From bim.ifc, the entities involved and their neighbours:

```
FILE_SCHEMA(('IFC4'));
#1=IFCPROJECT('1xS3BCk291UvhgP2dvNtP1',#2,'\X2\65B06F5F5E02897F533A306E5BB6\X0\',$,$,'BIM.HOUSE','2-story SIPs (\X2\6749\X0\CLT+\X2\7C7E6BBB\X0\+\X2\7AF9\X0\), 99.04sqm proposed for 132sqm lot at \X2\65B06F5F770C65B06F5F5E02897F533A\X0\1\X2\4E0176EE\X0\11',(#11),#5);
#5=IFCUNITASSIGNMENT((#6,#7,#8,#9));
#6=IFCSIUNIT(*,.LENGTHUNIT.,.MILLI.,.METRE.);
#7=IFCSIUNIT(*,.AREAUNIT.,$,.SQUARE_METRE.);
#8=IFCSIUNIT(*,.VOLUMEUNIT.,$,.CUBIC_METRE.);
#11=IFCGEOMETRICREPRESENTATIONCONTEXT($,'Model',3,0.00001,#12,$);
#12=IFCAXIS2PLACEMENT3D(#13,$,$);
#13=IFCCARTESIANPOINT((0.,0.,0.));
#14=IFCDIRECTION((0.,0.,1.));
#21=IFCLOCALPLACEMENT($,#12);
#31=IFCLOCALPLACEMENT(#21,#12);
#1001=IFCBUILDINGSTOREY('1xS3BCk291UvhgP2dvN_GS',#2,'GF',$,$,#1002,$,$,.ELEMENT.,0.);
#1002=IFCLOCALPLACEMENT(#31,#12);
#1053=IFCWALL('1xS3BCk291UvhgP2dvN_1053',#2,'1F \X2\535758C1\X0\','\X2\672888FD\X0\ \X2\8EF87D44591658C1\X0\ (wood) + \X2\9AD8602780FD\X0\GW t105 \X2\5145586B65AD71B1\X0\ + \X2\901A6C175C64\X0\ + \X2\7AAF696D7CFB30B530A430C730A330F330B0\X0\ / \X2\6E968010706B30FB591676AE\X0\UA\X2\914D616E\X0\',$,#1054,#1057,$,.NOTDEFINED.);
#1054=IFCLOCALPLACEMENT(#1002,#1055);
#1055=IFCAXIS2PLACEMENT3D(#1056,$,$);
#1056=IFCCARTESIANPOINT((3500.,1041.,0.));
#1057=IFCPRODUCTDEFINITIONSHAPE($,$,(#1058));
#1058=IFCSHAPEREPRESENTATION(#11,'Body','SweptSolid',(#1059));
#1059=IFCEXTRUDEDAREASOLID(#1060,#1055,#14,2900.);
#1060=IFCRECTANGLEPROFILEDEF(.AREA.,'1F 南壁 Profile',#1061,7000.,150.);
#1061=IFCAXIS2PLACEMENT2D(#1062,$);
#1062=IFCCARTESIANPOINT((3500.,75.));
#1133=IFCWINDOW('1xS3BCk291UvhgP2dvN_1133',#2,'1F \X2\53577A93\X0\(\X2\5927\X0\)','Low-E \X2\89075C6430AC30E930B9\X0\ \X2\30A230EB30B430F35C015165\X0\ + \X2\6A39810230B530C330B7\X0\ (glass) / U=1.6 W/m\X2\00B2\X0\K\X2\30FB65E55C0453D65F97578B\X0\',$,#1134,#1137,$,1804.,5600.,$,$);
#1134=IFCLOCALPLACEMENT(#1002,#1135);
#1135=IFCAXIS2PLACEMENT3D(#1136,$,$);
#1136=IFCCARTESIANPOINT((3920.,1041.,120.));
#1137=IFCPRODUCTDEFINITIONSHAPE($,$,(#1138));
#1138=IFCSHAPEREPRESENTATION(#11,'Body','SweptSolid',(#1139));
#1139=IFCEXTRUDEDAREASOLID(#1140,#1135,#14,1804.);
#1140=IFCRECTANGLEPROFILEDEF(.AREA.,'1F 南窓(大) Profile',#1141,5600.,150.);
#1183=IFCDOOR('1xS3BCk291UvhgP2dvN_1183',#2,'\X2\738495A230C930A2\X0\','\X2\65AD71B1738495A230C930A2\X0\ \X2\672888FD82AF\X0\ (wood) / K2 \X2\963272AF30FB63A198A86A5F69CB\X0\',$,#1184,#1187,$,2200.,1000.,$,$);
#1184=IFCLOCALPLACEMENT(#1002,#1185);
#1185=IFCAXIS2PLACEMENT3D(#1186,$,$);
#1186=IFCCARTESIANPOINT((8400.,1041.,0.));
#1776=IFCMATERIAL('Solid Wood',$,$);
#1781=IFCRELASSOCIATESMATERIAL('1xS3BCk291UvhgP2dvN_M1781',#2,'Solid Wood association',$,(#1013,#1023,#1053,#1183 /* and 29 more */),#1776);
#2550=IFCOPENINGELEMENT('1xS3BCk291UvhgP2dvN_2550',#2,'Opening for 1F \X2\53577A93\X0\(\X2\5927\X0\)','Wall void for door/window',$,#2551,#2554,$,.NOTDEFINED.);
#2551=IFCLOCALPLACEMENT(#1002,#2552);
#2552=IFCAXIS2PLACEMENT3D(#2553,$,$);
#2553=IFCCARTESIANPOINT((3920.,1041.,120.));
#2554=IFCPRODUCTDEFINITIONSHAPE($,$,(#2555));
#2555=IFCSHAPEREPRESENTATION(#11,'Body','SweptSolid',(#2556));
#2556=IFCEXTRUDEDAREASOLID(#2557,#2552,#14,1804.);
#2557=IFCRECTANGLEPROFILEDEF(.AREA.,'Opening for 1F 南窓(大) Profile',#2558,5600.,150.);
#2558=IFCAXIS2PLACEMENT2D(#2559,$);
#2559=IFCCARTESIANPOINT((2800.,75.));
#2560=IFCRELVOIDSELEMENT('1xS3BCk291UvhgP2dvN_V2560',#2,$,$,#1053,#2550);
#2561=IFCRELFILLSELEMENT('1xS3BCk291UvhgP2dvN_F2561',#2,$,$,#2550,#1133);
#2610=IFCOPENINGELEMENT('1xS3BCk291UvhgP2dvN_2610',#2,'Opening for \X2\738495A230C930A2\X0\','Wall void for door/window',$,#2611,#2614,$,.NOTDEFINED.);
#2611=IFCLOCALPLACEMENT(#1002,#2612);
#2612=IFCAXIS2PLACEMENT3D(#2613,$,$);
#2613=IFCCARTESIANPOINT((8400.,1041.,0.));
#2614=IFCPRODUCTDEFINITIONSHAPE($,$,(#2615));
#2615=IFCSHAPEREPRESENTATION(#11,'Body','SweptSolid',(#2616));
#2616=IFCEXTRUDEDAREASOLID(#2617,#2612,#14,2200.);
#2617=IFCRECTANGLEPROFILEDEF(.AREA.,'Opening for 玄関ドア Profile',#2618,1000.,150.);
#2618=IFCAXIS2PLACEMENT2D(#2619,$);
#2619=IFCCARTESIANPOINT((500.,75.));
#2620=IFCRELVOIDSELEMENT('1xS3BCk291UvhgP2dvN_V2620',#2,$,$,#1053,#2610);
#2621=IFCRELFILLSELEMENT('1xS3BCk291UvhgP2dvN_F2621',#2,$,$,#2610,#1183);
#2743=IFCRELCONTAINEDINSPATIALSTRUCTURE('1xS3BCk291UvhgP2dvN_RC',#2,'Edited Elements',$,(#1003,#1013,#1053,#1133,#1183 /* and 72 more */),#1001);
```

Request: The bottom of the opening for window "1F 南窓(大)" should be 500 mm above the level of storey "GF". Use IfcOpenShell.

```python
import numpy as np
import ifcopenshell
import ifcopenshell.api.geometry
import ifcopenshell.geom
import ifcopenshell.util.element
import ifcopenshell.util.placement
import ifcopenshell.util.shape
import ifcopenshell.util.unit

model = ifcopenshell.open("bim.ifc")
unit_scale = ifcopenshell.util.unit.calculate_unit_scale(model)

window = model.by_guid("1xS3BCk291UvhgP2dvN_1133")
opening = window.FillsVoids[0].RelatingOpeningElement
storey = ifcopenshell.util.element.get_container(window, ifc_class="IfcBuildingStorey")
level = ifcopenshell.util.placement.get_local_placement(storey.ObjectPlacement)[2, 3]

# The opening's origin need not be at the sill, so measure its lowest point.
shape = ifcopenshell.geom.create_shape(ifcopenshell.geom.settings(), opening)
bottom = ifcopenshell.util.shape.get_shape_bottom_elevation(shape, shape.geometry) / unit_scale
dz = level + 0.5 / unit_scale - bottom

shift = np.array([0.0, 0.0, dz])
# The window is not placed relative to its opening, so move both.
for product in (opening, window):
    matrix = ifcopenshell.util.placement.get_local_placement(product.ObjectPlacement)
    matrix[:3, 3] += shift
    ifcopenshell.api.geometry.edit_object_placement(model, product=product, matrix=matrix, is_si=False)

print(f"moved by {dz * unit_scale:+.3f} m")

model.write("bim_v2.ifc")
```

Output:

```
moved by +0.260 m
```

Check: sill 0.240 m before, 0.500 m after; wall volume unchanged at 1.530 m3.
